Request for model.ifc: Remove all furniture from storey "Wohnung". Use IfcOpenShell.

First a look at what the model holds.

```python
import ifcopenshell
import ifcopenshell.util.element

model = ifcopenshell.open("model.ifc")
print(model.schema)
storey = next(s for s in model.by_type("IfcBuildingStorey") if s.Name == "Wohnung")
furniture = [e for e in ifcopenshell.util.element.get_decomposition(storey) if e.is_a("IfcFurnishingElement")]
seen = {}
for e in furniture:
    element_type = ifcopenshell.util.element.get_type(e)
    name = element_type.Name if element_type not in (None, e) else None
    seen[name] = seen.get(name, 0) + 1
for name, count in sorted(seen.items(), key=str):
    print(count, "x", name)
```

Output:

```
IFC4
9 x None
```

```python
import ifcopenshell
import ifcopenshell.api.root
import ifcopenshell.util.element

model = ifcopenshell.open("model.ifc")

storey = next(s for s in model.by_type("IfcBuildingStorey") if s.Name == "Wohnung")
furniture = [e for e in ifcopenshell.util.element.get_decomposition(storey) if e.is_a("IfcFurnishingElement")]

for e in furniture:
    ifcopenshell.api.root.remove_product(model, product=e)
print(len(furniture), "removed")

model.write("model_updated.ifc")
```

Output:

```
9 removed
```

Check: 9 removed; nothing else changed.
